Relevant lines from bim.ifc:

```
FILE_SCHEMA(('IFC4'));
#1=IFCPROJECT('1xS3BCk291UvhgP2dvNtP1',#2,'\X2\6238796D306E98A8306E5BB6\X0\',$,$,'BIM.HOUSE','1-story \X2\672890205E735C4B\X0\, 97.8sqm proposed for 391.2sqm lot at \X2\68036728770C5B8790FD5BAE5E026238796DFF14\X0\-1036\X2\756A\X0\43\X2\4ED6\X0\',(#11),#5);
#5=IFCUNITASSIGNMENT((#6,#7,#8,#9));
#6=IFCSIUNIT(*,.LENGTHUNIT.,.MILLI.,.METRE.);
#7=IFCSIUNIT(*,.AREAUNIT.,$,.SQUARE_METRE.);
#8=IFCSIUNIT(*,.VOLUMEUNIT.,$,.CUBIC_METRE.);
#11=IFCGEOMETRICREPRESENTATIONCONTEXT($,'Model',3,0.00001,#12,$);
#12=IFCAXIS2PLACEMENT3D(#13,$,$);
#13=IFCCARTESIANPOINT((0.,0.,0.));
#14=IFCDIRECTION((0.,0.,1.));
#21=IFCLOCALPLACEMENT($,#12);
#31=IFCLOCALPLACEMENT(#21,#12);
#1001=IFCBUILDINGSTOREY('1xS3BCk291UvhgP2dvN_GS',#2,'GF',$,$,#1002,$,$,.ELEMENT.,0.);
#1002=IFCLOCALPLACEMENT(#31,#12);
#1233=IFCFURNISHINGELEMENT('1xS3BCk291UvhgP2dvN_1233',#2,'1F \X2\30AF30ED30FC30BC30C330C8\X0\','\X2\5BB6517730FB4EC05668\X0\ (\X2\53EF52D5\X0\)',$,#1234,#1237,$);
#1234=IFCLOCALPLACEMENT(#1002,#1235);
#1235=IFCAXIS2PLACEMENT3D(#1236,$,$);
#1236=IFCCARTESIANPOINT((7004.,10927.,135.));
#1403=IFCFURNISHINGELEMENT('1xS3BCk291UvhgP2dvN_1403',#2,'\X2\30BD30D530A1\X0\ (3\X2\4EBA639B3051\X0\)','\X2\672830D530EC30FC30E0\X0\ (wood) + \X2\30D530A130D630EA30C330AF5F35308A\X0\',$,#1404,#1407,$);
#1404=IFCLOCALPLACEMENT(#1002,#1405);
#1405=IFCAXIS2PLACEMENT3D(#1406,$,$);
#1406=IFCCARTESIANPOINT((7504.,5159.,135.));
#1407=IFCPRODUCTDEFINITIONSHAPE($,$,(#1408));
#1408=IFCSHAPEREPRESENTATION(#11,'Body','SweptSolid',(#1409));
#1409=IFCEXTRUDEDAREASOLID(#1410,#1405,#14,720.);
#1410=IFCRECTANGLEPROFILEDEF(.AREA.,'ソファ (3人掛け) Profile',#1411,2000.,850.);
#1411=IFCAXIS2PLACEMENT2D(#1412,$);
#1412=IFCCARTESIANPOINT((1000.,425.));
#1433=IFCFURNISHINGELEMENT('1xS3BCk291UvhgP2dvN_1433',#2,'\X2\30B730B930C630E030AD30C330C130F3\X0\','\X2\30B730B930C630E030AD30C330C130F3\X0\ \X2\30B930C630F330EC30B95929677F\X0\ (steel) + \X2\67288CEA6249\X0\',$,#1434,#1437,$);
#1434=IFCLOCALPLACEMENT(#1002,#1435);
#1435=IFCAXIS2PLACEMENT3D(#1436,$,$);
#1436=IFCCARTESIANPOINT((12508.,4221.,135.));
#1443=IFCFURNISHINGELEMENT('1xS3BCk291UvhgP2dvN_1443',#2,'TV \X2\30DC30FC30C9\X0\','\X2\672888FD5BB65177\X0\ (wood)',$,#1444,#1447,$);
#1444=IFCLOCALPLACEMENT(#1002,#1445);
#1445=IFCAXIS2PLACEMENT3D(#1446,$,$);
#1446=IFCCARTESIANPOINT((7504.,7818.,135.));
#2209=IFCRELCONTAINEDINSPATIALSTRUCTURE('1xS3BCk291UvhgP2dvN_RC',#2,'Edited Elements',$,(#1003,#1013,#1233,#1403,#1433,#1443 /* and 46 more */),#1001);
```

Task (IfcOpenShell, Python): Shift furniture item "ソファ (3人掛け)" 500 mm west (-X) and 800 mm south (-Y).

```python
import ifcopenshell
import ifcopenshell.api.geometry
import ifcopenshell.util.placement
import ifcopenshell.util.unit

model = ifcopenshell.open("bim.ifc")
unit_scale = ifcopenshell.util.unit.calculate_unit_scale(model)

item = model.by_guid("1xS3BCk291UvhgP2dvN_1403")
matrix = ifcopenshell.util.placement.get_local_placement(item.ObjectPlacement)
matrix[0, 3] -= 0.5 / unit_scale
matrix[1, 3] -= 0.8 / unit_scale
ifcopenshell.api.geometry.edit_object_placement(model, product=item, matrix=matrix, is_si=False)

print(ifcopenshell.util.placement.get_local_placement(item.ObjectPlacement).round(3) + 0.0)

model.write("bim-out.ifc")
```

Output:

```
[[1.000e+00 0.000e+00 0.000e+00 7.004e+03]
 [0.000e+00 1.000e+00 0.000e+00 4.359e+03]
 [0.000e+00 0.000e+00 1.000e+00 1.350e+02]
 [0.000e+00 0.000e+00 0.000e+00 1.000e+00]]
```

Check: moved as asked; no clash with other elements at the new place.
